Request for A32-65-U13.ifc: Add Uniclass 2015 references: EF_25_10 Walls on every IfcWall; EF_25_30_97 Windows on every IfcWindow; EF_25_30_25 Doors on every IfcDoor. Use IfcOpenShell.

First a look at what the model holds.

```python
import ifcopenshell

model = ifcopenshell.open("A32-65-U13.ifc")
print(model.schema)
print("classifications:", [c.Name for c in model.by_type("IfcClassification")])
for ifc_class in ("IfcDoor", "IfcRoof", "IfcStair", "IfcWall", "IfcWindow"):
    print(ifc_class, len(model.by_type(ifc_class)))
```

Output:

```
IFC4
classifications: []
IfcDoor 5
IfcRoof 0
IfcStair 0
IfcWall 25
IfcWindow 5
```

```python
import ifcopenshell
import ifcopenshell.api.classification

model = ifcopenshell.open("A32-65-U13.ifc")

system = ifcopenshell.api.classification.add_classification(model, classification="Uniclass 2015")

codes = {
    "IfcWall": ("EF_25_10", "Walls"),
    "IfcWindow": ("EF_25_30_97", "Windows"),
    "IfcDoor": ("EF_25_30_25", "Doors"),
}
for ifc_class, (code, name) in codes.items():
    products = model.by_type(ifc_class)
    ifcopenshell.api.classification.add_reference(
        model, products=products, classification=system, identification=code, name=name
    )
    print(code, len(products))

model.write("A32-65-U13_rev.ifc")
```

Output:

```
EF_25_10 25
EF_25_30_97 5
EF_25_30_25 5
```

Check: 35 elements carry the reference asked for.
